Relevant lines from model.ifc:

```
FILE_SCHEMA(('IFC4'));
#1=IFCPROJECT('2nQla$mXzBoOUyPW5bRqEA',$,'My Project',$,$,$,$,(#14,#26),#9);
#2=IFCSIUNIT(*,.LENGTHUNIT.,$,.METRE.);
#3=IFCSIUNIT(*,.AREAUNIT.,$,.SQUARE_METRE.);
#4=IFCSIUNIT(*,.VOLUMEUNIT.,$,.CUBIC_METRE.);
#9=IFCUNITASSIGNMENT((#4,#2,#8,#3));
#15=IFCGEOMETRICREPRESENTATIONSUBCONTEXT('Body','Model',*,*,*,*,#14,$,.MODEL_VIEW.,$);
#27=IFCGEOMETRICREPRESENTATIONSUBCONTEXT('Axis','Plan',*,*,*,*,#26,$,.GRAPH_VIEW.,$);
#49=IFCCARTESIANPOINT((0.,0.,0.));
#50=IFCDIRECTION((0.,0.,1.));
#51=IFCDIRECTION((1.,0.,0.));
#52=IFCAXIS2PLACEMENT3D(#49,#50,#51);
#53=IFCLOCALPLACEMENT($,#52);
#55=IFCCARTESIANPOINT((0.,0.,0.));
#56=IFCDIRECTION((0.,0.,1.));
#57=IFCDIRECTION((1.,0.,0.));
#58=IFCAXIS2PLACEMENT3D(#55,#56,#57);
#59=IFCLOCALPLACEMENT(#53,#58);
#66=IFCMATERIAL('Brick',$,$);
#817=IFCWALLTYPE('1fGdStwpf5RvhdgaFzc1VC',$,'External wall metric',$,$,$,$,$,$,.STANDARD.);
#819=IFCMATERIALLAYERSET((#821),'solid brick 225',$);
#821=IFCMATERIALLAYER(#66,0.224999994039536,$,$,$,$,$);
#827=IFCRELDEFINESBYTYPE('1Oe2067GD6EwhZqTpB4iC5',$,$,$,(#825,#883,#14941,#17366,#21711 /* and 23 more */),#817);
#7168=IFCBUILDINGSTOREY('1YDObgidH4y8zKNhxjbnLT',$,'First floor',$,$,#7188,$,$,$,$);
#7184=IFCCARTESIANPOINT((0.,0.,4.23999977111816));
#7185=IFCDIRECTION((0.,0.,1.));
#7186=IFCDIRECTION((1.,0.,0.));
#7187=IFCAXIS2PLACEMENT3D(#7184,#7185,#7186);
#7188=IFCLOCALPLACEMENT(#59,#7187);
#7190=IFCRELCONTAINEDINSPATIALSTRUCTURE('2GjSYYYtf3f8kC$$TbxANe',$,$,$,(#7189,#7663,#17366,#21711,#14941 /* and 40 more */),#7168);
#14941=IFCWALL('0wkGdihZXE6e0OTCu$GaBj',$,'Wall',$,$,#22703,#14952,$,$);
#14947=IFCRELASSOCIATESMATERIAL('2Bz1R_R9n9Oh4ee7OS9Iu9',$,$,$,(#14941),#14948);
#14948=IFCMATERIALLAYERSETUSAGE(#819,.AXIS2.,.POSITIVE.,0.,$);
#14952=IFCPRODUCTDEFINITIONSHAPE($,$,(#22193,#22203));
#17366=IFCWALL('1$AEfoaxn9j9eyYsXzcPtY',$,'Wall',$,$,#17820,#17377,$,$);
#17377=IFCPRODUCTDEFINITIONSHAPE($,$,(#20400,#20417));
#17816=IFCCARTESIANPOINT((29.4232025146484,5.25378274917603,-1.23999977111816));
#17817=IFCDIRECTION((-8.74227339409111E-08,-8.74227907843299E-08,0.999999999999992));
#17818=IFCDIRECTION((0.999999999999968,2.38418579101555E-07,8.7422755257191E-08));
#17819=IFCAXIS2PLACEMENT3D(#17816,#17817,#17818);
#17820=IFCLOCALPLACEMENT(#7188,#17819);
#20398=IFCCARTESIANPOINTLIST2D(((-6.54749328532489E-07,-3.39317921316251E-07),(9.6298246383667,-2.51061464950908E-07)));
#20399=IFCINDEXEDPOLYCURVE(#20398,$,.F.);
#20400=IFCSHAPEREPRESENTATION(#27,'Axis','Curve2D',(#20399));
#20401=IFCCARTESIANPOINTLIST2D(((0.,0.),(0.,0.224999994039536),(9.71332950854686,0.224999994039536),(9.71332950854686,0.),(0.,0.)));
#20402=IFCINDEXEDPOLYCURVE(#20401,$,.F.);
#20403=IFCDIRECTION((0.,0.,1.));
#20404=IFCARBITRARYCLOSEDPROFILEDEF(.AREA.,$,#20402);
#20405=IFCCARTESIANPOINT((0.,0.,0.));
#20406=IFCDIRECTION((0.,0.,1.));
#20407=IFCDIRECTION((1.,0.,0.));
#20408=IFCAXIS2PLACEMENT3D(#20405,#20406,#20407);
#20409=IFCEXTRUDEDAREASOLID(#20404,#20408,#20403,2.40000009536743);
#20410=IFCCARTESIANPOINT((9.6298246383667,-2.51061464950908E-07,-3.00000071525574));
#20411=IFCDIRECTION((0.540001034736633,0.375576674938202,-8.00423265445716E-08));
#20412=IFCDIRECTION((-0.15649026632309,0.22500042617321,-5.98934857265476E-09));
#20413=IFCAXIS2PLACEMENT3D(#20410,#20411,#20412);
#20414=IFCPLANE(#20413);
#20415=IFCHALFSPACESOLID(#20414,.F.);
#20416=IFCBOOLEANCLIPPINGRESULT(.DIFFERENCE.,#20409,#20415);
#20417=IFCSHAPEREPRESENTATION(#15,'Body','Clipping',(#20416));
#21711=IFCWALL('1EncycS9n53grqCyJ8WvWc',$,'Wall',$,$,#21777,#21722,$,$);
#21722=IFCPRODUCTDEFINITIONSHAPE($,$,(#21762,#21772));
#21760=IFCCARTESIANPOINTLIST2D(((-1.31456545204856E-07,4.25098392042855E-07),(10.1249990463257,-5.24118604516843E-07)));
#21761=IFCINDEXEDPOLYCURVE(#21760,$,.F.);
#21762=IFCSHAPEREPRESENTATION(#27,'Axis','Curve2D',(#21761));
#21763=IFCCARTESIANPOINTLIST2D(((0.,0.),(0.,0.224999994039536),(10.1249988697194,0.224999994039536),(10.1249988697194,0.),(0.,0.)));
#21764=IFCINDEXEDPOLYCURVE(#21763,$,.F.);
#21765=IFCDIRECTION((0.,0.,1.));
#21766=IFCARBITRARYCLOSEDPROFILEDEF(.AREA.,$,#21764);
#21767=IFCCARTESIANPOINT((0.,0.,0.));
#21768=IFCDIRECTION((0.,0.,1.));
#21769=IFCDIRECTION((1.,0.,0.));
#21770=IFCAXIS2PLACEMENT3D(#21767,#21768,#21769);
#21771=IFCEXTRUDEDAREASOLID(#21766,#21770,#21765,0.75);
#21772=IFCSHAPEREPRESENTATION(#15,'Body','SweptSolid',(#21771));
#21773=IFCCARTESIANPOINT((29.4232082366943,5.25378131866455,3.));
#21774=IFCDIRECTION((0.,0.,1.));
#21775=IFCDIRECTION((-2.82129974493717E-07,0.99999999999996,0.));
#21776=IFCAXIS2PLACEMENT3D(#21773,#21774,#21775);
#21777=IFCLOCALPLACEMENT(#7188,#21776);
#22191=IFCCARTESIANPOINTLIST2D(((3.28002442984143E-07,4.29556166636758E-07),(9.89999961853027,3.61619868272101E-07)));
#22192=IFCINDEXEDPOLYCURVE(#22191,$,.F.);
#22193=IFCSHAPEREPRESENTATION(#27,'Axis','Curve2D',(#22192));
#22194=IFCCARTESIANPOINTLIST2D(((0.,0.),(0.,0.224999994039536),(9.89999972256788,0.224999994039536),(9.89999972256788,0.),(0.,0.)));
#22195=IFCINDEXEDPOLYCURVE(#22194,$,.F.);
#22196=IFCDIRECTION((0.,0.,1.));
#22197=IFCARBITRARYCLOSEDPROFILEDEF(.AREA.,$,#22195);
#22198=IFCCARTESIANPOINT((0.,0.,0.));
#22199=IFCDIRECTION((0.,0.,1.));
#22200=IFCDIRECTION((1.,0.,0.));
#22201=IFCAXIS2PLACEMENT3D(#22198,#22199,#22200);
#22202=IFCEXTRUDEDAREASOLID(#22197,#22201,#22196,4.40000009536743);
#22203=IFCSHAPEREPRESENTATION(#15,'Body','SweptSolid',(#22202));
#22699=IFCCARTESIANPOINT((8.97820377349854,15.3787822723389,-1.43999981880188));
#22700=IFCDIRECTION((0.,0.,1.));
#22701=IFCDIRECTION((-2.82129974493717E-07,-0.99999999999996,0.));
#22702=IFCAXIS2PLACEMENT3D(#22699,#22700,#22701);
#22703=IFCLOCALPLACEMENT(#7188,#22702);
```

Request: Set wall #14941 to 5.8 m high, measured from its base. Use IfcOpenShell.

```python
import ifcopenshell
import ifcopenshell.geom
import ifcopenshell.util.representation
import ifcopenshell.util.shape
import ifcopenshell.util.unit

model = ifcopenshell.open("model.ifc")
unit_scale = ifcopenshell.util.unit.calculate_unit_scale(model)
settings = ifcopenshell.geom.settings()


def volume(element):
    """Net volume in cubic metres, openings subtracted."""
    shape = ifcopenshell.geom.create_shape(settings, element)
    return ifcopenshell.util.shape.get_volume(shape.geometry)


wall = model.by_id(14941)
before = volume(wall)

body = ifcopenshell.util.representation.get_representation(wall, "Model", "Body")
solid = body.Items[0]
old_height = solid.Depth
solid.Depth = 5.8 / unit_scale
after = volume(wall)

print(f"height {old_height:g} -> {solid.Depth:g}, volume {before:.3f} -> {after:.3f} m3")

model.write("model_v2.ifc")
```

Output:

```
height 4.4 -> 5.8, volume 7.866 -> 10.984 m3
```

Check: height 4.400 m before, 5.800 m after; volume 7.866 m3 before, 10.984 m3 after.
